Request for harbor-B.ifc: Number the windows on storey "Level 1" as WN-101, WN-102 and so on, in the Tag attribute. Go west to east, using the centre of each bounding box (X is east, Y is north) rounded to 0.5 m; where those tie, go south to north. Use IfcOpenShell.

First a look at what the model holds.

```python
import ifcopenshell
import ifcopenshell.util.element
import ifcopenshell.util.placement

model = ifcopenshell.open("harbor-B.ifc")
print(model.schema)
storey = next(s for s in model.by_type("IfcBuildingStorey") if s.Name == "Level 1")
windows = [e for e in ifcopenshell.util.element.get_decomposition(storey) if e.is_a("IfcWindow")]
for e in sorted(windows, key=lambda e: e.id()):
    origin = ifcopenshell.util.placement.get_local_placement(e.ObjectPlacement)[:3, 3]
    print(e.id(), e.Tag, e.Name, origin.round(2) + 0.0, sep=" | ")
```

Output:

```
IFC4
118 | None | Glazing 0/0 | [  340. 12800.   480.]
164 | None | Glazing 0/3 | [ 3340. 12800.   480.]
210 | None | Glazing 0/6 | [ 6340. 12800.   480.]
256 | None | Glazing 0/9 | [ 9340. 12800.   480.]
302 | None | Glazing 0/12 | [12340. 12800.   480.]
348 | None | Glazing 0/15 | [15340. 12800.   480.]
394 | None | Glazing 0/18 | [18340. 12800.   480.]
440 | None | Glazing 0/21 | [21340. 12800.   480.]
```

```python
import ifcopenshell
import ifcopenshell.geom
import ifcopenshell.util.element
import ifcopenshell.util.shape

model = ifcopenshell.open("harbor-B.ifc")
settings = ifcopenshell.geom.settings()
settings.set("use-world-coords", True)


def centre(element):
    shape = ifcopenshell.geom.create_shape(settings, element)
    return ifcopenshell.util.shape.get_bbox_centroid(shape.geometry)


storey = next(s for s in model.by_type("IfcBuildingStorey") if s.Name == "Level 1")
windows = [e for e in ifcopenshell.util.element.get_decomposition(storey) if e.is_a("IfcWindow")]

# Insertion points can sit at a corner or the storey origin, so sort by the geometry (in metres).
centres = {e: centre(e) for e in windows}
windows.sort(key=lambda e: (round(centres[e][0] / 0.5), centres[e][1]))

for i, e in enumerate(windows, start=1):
    number = f"WN-1{i:02d}"
    e.Tag = number
    print(e.id(), number)

model.write("harbor-B_edited.ifc")
```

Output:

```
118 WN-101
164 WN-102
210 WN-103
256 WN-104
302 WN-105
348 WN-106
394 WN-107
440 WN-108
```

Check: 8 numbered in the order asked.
